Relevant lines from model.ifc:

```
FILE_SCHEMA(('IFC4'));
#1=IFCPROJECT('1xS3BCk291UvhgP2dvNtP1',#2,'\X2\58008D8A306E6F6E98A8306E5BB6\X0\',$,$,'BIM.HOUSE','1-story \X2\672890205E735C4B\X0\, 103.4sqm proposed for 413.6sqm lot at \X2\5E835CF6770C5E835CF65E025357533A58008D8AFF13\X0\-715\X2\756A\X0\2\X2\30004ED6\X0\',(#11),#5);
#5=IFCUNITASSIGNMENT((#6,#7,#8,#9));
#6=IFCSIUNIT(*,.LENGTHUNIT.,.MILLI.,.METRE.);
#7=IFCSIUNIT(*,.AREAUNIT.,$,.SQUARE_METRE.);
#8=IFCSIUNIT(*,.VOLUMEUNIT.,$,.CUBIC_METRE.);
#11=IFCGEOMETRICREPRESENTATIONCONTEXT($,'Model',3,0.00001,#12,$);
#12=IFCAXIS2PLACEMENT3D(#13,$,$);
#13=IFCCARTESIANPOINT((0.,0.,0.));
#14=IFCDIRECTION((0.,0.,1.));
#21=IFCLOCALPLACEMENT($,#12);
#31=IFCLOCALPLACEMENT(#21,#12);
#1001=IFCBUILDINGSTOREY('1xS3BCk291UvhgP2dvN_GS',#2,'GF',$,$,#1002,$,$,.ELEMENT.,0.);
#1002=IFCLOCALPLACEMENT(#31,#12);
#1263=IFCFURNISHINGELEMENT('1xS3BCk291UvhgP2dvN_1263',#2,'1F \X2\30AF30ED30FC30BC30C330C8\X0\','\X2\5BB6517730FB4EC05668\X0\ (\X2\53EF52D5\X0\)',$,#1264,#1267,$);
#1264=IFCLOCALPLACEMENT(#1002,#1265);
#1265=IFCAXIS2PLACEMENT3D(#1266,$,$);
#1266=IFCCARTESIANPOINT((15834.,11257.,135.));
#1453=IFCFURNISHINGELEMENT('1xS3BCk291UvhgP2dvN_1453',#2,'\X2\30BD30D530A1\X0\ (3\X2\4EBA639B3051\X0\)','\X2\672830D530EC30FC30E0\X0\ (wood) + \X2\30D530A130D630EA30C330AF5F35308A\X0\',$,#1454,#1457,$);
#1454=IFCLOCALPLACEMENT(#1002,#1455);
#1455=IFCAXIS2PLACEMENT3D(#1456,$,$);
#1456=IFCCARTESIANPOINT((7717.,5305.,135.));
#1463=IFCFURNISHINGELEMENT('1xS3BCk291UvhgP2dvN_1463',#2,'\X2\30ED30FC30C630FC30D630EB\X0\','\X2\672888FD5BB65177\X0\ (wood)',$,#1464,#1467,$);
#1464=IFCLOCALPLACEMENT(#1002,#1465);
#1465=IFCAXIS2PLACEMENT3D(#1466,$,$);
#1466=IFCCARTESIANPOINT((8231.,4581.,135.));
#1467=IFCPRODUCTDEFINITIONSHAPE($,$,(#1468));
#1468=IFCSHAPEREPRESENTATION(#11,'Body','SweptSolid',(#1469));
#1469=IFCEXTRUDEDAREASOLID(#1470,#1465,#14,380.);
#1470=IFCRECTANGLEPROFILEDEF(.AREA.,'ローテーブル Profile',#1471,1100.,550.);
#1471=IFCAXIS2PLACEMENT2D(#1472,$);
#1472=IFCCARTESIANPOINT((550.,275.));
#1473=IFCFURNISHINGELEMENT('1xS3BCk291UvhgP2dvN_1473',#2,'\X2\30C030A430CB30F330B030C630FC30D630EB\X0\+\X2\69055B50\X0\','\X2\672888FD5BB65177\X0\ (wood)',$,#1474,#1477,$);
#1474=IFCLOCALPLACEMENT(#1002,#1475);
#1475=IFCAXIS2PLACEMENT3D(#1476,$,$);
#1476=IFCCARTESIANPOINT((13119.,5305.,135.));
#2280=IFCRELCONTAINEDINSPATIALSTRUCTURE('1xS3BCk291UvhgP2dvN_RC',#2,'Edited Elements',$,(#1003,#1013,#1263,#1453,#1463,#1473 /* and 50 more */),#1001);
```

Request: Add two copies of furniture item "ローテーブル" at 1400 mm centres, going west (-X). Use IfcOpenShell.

```python
import numpy as np
import ifcopenshell
import ifcopenshell.api.geometry
import ifcopenshell.api.root
import ifcopenshell.util.element
import ifcopenshell.util.placement

model = ifcopenshell.open("model.ifc")


def reuse_history(source, copy):
    """copy_class also copies each property set's owner history, people and application; keep the originals."""
    for rel in copy.IsDefinedBy:
        if rel.is_a("IfcRelDefinesByProperties") and (history := rel.RelatingPropertyDefinition.OwnerHistory):
            rel.RelatingPropertyDefinition.OwnerHistory = source.OwnerHistory
            ifcopenshell.util.element.remove_deep2(model, history)


source = model.by_guid("1xS3BCk291UvhgP2dvN_1463")
base = ifcopenshell.util.placement.get_local_placement(source.ObjectPlacement)
step = np.array([-1.0, 0.0, 0.0]) * 1400.0

for i in range(1, 3):
    copy = ifcopenshell.api.root.copy_class(model, product=source)
    copy.Representation = ifcopenshell.util.element.copy_deep(
        model, source.Representation, exclude=["IfcGeometricRepresentationContext", "IfcRepresentationMap"]
    )
    reuse_history(source, copy)
    matrix = base.copy()
    matrix[:3, 3] += i * step
    print("added at", matrix[:3, 3].round(3) + 0.0)
    ifcopenshell.api.geometry.edit_object_placement(model, product=copy, matrix=matrix, is_si=False)

model.write("model_edited.ifc")
```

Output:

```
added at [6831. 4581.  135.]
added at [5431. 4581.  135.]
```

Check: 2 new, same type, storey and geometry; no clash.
